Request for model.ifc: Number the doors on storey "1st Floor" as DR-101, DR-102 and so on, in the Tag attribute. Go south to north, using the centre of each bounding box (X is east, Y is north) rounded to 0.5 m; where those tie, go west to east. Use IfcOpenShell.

First a look at what the model holds.

```python
import ifcopenshell
import ifcopenshell.util.element
import ifcopenshell.util.placement

model = ifcopenshell.open("model.ifc")
print(model.schema)
storey = next(s for s in model.by_type("IfcBuildingStorey") if s.Name == "1st Floor")
doors = [e for e in ifcopenshell.util.element.get_decomposition(storey) if e.is_a("IfcDoor")]
for e in sorted(doors, key=lambda e: e.id()):
    origin = ifcopenshell.util.placement.get_local_placement(e.ObjectPlacement)[:3, 3]
    print(e.id(), e.Tag, e.Name, origin.round(2) + 0.0, sep=" | ")
```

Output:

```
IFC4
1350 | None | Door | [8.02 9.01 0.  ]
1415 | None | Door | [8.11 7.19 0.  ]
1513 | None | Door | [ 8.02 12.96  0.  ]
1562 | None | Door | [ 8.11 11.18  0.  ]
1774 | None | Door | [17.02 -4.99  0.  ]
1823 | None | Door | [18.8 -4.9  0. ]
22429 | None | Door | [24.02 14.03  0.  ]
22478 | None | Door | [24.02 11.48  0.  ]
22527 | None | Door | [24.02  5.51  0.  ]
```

```python
import ifcopenshell
import ifcopenshell.geom
import ifcopenshell.util.element
import ifcopenshell.util.shape

model = ifcopenshell.open("model.ifc")
settings = ifcopenshell.geom.settings()
settings.set("use-world-coords", True)


def centre(element):
    shape = ifcopenshell.geom.create_shape(settings, element)
    return ifcopenshell.util.shape.get_bbox_centroid(shape.geometry)


storey = next(s for s in model.by_type("IfcBuildingStorey") if s.Name == "1st Floor")
doors = [e for e in ifcopenshell.util.element.get_decomposition(storey) if e.is_a("IfcDoor")]

# Insertion points can sit at a corner or the storey origin, so sort by the geometry (in metres).
centres = {e: centre(e) for e in doors}
doors.sort(key=lambda e: (round(centres[e][1] / 0.5), centres[e][0]))

for i, e in enumerate(doors, start=1):
    number = f"DR-1{i:02d}"
    e.Tag = number
    print(e.id(), number)

model.write("model_edited.ifc")
```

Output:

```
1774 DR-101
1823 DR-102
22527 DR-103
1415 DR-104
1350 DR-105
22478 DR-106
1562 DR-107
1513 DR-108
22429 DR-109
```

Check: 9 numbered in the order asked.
